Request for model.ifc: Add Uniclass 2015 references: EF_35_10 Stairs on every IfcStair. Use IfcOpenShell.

First a look at what the model holds.

```python
import ifcopenshell

model = ifcopenshell.open("model.ifc")
print(model.schema)
print("classifications:", [c.Name for c in model.by_type("IfcClassification")])
for ifc_class in ("IfcDoor", "IfcRoof", "IfcStair", "IfcWall", "IfcWindow"):
    print(ifc_class, len(model.by_type(ifc_class)))
```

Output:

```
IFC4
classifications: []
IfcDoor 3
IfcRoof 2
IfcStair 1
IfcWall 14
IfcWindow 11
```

```python
import ifcopenshell
import ifcopenshell.api.classification

model = ifcopenshell.open("model.ifc")

system = ifcopenshell.api.classification.add_classification(model, classification="Uniclass 2015")

codes = {
    "IfcStair": ("EF_35_10", "Stairs"),
}
for ifc_class, (code, name) in codes.items():
    products = model.by_type(ifc_class)
    ifcopenshell.api.classification.add_reference(
        model, products=products, classification=system, identification=code, name=name
    )
    print(code, len(products))

model.write("model_edited.ifc")
```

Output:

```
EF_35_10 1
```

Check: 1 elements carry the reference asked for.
